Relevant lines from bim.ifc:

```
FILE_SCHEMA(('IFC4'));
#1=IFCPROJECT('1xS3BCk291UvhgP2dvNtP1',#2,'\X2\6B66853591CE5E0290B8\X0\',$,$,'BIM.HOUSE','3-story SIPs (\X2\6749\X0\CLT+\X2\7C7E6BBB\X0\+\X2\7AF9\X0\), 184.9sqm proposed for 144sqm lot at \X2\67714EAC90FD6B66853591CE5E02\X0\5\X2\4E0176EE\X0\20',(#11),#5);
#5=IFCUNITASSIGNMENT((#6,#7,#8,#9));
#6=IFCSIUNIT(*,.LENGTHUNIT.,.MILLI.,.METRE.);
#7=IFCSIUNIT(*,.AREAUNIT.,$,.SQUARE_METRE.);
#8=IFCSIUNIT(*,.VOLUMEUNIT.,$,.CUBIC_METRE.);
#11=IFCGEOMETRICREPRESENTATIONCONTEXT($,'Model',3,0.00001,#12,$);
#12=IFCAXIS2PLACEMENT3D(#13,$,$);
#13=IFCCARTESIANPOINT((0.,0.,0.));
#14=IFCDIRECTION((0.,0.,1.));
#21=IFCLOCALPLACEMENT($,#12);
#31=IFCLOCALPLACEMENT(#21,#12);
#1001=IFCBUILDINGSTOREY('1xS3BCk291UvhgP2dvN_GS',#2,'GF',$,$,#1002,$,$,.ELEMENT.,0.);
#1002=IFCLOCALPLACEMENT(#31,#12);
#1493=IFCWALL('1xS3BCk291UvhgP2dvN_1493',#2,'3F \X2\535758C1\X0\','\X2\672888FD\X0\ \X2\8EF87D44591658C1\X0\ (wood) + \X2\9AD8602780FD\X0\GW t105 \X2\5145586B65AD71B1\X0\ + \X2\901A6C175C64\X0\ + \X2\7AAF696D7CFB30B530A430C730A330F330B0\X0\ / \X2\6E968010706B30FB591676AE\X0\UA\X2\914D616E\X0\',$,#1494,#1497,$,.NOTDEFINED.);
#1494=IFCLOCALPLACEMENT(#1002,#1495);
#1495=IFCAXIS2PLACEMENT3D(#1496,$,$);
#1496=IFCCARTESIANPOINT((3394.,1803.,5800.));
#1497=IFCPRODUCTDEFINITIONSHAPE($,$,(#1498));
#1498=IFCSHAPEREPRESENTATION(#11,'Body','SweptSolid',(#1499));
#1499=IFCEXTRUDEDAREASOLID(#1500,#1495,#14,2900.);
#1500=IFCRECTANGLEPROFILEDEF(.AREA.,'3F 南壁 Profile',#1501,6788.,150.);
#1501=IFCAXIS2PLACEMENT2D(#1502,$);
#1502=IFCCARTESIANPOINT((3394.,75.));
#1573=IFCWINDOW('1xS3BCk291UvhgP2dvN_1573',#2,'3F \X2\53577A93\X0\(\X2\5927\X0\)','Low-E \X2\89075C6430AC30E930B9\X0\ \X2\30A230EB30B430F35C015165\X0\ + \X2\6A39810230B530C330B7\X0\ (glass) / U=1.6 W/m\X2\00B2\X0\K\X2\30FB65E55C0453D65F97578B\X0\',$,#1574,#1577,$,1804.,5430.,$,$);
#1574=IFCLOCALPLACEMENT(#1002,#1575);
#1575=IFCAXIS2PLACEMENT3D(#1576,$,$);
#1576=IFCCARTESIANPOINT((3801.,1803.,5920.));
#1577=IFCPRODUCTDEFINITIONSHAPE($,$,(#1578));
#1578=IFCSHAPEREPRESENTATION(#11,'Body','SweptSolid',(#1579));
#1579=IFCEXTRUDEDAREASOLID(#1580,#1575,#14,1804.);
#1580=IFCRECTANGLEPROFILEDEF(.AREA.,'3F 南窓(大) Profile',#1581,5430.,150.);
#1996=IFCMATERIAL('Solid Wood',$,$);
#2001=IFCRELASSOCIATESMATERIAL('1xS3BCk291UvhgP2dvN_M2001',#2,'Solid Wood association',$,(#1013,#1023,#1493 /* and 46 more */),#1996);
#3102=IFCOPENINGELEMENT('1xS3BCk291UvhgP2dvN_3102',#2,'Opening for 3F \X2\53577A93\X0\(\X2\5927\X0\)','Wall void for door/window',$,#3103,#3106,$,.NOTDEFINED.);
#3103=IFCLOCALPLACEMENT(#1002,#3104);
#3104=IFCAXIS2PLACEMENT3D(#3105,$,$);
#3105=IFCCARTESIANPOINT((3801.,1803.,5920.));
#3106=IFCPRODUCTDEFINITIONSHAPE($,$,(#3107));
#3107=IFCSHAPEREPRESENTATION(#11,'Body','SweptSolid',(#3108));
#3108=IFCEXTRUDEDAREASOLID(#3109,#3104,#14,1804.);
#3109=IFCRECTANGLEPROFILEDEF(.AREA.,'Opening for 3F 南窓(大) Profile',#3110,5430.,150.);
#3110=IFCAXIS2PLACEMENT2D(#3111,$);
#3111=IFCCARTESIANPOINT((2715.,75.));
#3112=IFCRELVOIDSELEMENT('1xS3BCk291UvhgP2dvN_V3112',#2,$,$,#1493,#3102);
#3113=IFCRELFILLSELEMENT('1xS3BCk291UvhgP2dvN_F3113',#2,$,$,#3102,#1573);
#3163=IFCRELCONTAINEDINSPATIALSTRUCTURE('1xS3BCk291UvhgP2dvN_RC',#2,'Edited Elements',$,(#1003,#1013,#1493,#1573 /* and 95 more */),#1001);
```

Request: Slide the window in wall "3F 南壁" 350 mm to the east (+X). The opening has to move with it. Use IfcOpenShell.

```python
import ifcopenshell
import ifcopenshell.api.geometry
import ifcopenshell.util.placement
import ifcopenshell.util.unit

model = ifcopenshell.open("bim.ifc")
unit_scale = ifcopenshell.util.unit.calculate_unit_scale(model)

window = model.by_id(1573)
opening = window.FillsVoids[0].RelatingOpeningElement
wall = opening.VoidsElements[0].RelatingBuildingElement

wall_matrix = ifcopenshell.util.placement.get_local_placement(wall.ObjectPlacement)
shift = wall_matrix[:3, 0] * 0.35 / unit_scale
before = ifcopenshell.util.placement.get_local_placement(window.ObjectPlacement)[:3, 3].copy()

# The window is not placed relative to its opening, so move both.
for product in (opening, window):
    matrix = ifcopenshell.util.placement.get_local_placement(product.ObjectPlacement)
    matrix[:3, 3] += shift
    ifcopenshell.api.geometry.edit_object_placement(model, product=product, matrix=matrix, is_si=False)

after = ifcopenshell.util.placement.get_local_placement(window.ObjectPlacement)[:3, 3]
print("window moved by", (after - before).round(3) + 0.0)

model.write("bim_edited.ifc")
```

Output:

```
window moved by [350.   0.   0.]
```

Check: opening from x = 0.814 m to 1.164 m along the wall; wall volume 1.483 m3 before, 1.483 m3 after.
